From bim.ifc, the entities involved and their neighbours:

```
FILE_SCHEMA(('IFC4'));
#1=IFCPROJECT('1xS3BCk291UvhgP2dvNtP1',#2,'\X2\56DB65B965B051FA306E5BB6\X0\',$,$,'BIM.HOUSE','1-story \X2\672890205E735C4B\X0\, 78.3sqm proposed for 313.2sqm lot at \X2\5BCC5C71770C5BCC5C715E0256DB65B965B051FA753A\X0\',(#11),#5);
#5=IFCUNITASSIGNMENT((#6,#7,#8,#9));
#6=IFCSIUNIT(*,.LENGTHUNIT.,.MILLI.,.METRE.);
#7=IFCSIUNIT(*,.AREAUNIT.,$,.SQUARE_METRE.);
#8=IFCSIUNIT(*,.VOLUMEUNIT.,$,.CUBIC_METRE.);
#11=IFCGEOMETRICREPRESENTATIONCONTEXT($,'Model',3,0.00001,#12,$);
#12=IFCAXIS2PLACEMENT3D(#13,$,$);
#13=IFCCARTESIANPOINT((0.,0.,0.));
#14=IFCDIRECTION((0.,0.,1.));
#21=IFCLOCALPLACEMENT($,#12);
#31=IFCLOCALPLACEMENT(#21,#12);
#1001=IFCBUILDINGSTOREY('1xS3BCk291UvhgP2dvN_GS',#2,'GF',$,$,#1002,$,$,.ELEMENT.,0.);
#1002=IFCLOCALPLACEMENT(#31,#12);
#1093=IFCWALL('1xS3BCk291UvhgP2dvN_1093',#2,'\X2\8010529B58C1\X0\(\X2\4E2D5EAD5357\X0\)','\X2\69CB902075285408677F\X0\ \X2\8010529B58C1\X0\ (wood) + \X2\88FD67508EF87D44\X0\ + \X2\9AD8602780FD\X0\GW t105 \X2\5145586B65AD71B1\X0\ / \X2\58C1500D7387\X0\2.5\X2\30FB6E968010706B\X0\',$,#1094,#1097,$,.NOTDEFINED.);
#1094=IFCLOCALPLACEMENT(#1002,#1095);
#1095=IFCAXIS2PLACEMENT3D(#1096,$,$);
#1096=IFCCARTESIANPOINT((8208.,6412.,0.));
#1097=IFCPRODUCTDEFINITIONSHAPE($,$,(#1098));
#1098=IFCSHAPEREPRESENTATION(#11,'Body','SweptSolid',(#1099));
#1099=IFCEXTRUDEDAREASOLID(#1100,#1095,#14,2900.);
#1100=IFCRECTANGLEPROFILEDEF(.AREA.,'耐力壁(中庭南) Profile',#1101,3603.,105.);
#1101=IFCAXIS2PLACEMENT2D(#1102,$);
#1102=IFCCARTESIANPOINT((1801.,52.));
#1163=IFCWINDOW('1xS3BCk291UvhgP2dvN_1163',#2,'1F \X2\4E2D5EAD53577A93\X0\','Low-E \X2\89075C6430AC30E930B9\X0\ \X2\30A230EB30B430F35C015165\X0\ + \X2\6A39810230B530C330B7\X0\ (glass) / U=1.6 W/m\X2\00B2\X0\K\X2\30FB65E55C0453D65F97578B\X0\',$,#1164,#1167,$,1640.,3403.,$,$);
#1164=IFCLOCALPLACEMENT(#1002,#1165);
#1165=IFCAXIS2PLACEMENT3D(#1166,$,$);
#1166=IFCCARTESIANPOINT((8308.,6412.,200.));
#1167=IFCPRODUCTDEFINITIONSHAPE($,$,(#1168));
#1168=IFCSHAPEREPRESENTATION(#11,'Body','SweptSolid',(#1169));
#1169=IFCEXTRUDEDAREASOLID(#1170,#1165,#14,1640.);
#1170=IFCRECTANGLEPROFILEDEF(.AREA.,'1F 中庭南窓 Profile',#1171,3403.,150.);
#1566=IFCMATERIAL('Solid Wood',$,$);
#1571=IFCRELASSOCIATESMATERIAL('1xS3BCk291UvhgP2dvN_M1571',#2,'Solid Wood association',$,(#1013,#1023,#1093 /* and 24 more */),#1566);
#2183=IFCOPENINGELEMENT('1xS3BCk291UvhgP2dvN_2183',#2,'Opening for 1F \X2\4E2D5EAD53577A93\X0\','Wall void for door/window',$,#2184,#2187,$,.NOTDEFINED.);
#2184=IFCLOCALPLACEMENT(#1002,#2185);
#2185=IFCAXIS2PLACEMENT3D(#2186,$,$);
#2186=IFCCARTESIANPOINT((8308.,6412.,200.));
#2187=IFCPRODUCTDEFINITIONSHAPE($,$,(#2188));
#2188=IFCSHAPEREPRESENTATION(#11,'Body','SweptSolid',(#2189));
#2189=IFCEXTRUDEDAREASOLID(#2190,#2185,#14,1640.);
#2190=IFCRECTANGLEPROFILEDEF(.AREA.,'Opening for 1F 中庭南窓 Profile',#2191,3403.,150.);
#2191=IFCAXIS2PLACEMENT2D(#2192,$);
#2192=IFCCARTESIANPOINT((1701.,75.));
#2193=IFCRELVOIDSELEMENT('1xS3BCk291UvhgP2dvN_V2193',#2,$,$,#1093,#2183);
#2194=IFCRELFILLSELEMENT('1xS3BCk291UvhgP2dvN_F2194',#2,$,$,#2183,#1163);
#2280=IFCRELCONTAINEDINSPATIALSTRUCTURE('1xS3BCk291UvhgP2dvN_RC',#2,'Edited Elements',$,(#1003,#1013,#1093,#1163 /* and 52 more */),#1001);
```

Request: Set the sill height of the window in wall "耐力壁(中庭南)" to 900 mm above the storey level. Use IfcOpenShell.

```python
import numpy as np
import ifcopenshell
import ifcopenshell.api.geometry
import ifcopenshell.geom
import ifcopenshell.util.element
import ifcopenshell.util.placement
import ifcopenshell.util.shape
import ifcopenshell.util.unit

model = ifcopenshell.open("bim.ifc")
unit_scale = ifcopenshell.util.unit.calculate_unit_scale(model)

window = model.by_guid("1xS3BCk291UvhgP2dvN_1163")
opening = window.FillsVoids[0].RelatingOpeningElement
storey = ifcopenshell.util.element.get_container(window, ifc_class="IfcBuildingStorey")
level = ifcopenshell.util.placement.get_local_placement(storey.ObjectPlacement)[2, 3]

# The opening's origin need not be at the sill, so measure its lowest point.
shape = ifcopenshell.geom.create_shape(ifcopenshell.geom.settings(), opening)
bottom = ifcopenshell.util.shape.get_shape_bottom_elevation(shape, shape.geometry) / unit_scale
dz = level + 900.0 - bottom

shift = np.array([0.0, 0.0, dz])
# The window is not placed relative to its opening, so move both.
for product in (opening, window):
    matrix = ifcopenshell.util.placement.get_local_placement(product.ObjectPlacement)
    matrix[:3, 3] += shift
    ifcopenshell.api.geometry.edit_object_placement(model, product=product, matrix=matrix, is_si=False)

print(f"moved by {dz * unit_scale:+.3f} m")

model.write("bim_edited.ifc")
```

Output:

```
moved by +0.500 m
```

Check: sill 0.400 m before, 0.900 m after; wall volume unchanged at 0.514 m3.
